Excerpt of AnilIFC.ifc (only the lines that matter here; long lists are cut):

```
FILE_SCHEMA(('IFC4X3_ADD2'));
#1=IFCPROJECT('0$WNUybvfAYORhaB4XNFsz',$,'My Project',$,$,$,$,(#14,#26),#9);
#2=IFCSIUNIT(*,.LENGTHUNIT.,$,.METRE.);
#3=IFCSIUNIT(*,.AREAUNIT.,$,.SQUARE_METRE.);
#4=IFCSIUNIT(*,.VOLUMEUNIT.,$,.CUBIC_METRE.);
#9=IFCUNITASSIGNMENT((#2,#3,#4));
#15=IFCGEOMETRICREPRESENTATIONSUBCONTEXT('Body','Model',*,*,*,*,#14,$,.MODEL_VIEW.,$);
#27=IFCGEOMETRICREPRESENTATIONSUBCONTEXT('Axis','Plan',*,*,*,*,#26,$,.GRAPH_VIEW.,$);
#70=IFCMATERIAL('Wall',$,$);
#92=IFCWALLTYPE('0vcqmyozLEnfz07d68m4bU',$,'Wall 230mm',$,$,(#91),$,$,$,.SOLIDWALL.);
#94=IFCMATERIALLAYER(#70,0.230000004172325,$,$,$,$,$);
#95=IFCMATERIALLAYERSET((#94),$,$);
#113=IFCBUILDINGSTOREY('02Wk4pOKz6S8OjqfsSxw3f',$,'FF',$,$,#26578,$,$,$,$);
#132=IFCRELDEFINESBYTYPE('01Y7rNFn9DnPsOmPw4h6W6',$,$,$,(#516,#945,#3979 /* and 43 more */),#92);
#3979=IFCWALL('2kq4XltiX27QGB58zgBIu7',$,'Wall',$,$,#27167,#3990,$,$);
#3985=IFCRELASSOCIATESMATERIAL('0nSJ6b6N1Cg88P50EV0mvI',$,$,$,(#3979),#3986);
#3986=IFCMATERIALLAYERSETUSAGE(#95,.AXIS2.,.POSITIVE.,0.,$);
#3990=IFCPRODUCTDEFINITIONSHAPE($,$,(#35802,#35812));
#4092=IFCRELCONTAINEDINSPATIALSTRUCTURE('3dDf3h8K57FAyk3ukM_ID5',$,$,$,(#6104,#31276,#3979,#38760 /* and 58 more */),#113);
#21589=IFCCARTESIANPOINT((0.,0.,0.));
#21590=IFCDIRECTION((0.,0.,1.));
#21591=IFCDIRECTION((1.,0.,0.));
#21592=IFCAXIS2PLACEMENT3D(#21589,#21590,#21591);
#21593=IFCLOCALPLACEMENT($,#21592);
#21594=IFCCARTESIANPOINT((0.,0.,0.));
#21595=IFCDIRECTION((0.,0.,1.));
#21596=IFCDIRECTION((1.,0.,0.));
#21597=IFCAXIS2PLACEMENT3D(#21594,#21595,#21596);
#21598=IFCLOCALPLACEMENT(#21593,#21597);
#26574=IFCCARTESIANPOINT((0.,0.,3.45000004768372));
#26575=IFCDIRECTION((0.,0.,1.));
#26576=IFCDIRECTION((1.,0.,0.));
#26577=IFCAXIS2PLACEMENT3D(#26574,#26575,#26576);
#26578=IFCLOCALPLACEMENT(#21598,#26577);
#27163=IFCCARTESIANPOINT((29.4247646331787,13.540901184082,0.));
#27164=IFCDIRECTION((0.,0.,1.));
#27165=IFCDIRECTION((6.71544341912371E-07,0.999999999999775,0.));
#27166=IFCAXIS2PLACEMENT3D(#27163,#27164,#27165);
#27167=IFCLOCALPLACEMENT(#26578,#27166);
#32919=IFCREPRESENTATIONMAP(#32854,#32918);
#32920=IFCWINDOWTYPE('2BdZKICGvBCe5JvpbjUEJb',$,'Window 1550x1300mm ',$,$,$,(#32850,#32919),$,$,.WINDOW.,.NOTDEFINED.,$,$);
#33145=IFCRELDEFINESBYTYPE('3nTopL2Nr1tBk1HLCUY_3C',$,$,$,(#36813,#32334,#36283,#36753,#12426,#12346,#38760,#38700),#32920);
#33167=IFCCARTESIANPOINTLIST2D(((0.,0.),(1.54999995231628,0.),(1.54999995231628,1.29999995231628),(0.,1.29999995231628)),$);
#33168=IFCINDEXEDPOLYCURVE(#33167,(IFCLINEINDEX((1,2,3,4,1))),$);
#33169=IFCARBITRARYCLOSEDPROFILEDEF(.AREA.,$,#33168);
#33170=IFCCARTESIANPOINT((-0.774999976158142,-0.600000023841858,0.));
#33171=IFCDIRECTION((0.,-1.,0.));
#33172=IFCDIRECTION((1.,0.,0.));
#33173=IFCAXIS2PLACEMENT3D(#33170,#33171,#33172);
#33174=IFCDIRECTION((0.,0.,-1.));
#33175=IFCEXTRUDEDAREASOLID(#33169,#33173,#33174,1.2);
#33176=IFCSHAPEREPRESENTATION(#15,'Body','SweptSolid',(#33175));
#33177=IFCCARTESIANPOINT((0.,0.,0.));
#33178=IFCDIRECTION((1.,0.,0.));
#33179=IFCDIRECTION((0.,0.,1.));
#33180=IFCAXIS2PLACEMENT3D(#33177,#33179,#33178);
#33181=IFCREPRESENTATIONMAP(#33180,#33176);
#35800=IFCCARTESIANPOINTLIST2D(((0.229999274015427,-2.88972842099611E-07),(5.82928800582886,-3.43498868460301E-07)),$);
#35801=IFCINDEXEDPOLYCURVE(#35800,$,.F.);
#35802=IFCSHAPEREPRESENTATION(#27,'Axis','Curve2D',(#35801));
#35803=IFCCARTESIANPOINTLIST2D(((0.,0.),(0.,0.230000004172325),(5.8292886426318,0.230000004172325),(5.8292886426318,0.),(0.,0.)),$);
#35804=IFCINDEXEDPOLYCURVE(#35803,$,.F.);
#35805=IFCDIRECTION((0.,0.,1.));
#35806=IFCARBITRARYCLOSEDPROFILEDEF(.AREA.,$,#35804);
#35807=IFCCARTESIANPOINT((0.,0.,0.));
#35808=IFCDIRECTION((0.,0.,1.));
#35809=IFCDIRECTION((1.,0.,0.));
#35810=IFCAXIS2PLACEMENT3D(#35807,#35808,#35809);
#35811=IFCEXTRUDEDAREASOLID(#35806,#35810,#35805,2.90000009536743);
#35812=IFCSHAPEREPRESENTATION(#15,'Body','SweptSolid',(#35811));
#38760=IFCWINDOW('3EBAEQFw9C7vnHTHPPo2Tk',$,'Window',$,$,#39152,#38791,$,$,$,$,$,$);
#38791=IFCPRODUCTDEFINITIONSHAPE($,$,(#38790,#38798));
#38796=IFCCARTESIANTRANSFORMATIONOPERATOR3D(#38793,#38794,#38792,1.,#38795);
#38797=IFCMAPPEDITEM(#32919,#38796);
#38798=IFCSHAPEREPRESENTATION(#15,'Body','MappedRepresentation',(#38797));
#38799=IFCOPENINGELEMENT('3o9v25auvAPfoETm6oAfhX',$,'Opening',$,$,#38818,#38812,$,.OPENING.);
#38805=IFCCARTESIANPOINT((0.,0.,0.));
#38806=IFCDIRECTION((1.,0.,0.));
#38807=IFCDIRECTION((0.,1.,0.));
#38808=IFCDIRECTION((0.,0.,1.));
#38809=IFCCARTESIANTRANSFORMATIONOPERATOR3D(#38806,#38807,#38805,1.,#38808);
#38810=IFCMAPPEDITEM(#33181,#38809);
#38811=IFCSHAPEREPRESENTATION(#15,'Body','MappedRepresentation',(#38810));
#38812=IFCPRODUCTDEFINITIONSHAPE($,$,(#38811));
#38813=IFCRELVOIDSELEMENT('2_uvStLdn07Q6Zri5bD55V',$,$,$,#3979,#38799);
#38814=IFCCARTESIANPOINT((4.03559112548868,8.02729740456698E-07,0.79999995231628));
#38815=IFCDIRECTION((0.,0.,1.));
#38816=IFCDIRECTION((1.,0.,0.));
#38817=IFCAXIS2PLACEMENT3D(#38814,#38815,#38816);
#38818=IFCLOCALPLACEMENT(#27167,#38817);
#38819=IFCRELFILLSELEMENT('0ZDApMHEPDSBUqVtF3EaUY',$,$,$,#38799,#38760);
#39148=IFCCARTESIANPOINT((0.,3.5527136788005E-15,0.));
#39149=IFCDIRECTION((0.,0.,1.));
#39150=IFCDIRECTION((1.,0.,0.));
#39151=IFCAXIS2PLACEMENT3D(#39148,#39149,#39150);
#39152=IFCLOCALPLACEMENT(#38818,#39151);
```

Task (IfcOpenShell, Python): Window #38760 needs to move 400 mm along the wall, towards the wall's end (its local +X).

```python
import ifcopenshell
import ifcopenshell.api.geometry
import ifcopenshell.util.placement

model = ifcopenshell.open("AnilIFC.ifc")

window = model.by_guid("3EBAEQFw9C7vnHTHPPo2Tk")
opening = window.FillsVoids[0].RelatingOpeningElement
wall = opening.VoidsElements[0].RelatingBuildingElement

wall_matrix = ifcopenshell.util.placement.get_local_placement(wall.ObjectPlacement)
shift = wall_matrix[:3, 0] * 0.4
before = ifcopenshell.util.placement.get_local_placement(window.ObjectPlacement)[:3, 3].copy()

# The window is placed relative to its opening, so it follows when the opening moves.
matrix = ifcopenshell.util.placement.get_local_placement(opening.ObjectPlacement)
matrix[:3, 3] += shift
ifcopenshell.api.geometry.edit_object_placement(
    model, product=opening, matrix=matrix, is_si=False, should_transform_children=True
)

after = ifcopenshell.util.placement.get_local_placement(window.ObjectPlacement)[:3, 3]
print("window moved by", (after - before).round(3) + 0.0)

model.write("AnilIFC_v2.ifc")
```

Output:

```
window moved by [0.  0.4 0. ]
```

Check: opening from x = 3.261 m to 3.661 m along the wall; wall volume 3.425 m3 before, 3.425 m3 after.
